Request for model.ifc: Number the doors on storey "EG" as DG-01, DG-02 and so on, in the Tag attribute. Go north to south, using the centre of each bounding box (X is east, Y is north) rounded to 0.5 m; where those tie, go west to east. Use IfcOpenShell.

First a look at what the model holds.

```python
import ifcopenshell
import ifcopenshell.util.element
import ifcopenshell.util.placement

model = ifcopenshell.open("model.ifc")
print(model.schema)
storey = next(s for s in model.by_type("IfcBuildingStorey") if s.Name == "EG")
doors = [e for e in ifcopenshell.util.element.get_decomposition(storey) if e.is_a("IfcDoor")]
for e in sorted(doors, key=lambda e: e.id()):
    origin = ifcopenshell.util.placement.get_local_placement(e.ObjectPlacement)[:3, 3]
    print(e.id(), e.Tag, e.Name, origin.round(2) + 0.0, sep=" | ")
```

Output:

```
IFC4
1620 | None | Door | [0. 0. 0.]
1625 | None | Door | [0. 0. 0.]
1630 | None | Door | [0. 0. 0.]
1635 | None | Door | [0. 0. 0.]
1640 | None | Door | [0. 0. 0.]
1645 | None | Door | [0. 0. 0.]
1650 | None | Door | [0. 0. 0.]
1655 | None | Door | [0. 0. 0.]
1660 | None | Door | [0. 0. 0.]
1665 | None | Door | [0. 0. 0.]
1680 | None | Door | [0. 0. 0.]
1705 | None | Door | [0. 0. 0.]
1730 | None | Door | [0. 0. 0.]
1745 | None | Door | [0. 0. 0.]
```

```python
import ifcopenshell
import ifcopenshell.geom
import ifcopenshell.util.element
import ifcopenshell.util.shape

model = ifcopenshell.open("model.ifc")
settings = ifcopenshell.geom.settings()
settings.set("use-world-coords", True)


def centre(element):
    shape = ifcopenshell.geom.create_shape(settings, element)
    return ifcopenshell.util.shape.get_bbox_centroid(shape.geometry)


storey = next(s for s in model.by_type("IfcBuildingStorey") if s.Name == "EG")
doors = [e for e in ifcopenshell.util.element.get_decomposition(storey) if e.is_a("IfcDoor")]

# Insertion points can sit at a corner or the storey origin, so sort by the geometry (in metres).
centres = {e: centre(e) for e in doors}
doors.sort(key=lambda e: (-round(centres[e][1] / 0.5), centres[e][0]))

for i, e in enumerate(doors, start=1):
    number = f"DG-{i:02d}"
    e.Tag = number
    print(e.id(), number)

model.write("model-out.ifc")
```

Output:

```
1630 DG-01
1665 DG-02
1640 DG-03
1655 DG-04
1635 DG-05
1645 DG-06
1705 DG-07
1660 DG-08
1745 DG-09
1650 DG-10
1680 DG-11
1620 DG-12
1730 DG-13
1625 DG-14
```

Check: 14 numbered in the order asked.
